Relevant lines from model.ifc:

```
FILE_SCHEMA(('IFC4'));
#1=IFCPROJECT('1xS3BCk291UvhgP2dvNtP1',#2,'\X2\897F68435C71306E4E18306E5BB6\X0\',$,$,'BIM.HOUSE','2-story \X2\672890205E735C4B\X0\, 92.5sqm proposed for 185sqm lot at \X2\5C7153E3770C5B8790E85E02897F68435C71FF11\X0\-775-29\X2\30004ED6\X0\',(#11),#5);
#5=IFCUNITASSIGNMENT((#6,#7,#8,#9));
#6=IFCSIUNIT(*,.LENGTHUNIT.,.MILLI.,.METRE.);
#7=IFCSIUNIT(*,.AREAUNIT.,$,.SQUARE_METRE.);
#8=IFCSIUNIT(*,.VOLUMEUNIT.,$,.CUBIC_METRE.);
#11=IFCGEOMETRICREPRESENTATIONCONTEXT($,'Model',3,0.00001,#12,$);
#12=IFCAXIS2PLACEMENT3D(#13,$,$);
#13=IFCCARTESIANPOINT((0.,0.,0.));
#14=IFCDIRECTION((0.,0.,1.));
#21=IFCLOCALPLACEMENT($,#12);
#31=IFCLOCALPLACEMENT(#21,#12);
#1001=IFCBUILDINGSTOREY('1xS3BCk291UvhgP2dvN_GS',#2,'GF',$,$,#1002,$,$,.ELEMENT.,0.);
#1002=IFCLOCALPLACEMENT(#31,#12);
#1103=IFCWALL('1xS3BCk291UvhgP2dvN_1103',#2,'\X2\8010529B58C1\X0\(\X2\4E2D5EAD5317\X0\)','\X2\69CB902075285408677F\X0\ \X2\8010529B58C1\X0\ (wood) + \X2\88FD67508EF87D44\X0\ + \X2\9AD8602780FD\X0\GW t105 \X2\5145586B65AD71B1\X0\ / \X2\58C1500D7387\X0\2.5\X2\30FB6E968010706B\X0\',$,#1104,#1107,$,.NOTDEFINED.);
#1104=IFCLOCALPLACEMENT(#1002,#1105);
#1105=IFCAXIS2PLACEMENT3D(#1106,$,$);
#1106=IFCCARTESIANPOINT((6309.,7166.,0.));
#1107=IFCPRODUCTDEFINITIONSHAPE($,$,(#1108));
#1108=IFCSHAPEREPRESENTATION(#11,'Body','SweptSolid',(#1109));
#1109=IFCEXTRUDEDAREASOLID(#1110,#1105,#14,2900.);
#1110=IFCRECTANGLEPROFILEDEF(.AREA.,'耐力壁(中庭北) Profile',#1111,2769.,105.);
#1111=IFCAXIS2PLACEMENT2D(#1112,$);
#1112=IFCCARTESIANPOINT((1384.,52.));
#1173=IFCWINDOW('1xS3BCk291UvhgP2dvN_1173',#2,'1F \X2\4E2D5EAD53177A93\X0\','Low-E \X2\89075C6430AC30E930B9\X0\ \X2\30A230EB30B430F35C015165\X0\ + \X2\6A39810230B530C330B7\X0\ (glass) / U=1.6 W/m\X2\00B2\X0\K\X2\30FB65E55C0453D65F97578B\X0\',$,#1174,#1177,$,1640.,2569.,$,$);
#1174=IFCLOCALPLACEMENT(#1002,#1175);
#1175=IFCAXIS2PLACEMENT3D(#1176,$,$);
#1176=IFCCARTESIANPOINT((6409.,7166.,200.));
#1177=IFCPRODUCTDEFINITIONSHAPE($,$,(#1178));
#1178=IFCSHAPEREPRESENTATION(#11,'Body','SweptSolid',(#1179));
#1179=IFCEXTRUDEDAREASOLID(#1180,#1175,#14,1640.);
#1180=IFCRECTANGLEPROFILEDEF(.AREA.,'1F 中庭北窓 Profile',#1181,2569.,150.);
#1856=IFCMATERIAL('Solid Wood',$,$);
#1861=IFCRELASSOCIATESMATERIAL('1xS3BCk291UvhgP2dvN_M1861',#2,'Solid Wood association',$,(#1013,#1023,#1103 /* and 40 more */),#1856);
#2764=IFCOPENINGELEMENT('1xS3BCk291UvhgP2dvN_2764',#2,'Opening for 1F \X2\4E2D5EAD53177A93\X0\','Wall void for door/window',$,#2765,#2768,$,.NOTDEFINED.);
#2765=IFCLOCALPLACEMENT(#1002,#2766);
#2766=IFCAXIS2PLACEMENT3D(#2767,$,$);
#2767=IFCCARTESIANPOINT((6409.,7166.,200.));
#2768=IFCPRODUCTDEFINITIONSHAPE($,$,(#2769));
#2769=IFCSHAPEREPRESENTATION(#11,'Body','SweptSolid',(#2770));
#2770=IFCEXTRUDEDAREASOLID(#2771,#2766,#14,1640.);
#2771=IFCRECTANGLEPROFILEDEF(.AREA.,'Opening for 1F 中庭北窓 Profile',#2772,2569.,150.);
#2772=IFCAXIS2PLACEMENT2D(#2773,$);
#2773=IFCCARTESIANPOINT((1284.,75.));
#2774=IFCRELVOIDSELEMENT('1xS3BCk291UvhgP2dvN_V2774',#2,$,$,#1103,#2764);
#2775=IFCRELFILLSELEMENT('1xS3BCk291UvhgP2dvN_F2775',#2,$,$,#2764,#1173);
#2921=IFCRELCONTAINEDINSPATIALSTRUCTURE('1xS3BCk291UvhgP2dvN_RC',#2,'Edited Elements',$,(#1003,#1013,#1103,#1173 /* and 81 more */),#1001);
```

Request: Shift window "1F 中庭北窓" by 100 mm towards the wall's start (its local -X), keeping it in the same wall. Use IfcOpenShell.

```python
import ifcopenshell
import ifcopenshell.api.geometry
import ifcopenshell.util.placement

model = ifcopenshell.open("model.ifc")

window = model.by_guid("1xS3BCk291UvhgP2dvN_1173")
opening = window.FillsVoids[0].RelatingOpeningElement
wall = opening.VoidsElements[0].RelatingBuildingElement

wall_matrix = ifcopenshell.util.placement.get_local_placement(wall.ObjectPlacement)
shift = wall_matrix[:3, 0] * -100.0
before = ifcopenshell.util.placement.get_local_placement(window.ObjectPlacement)[:3, 3].copy()

# The window is not placed relative to its opening, so move both.
for product in (opening, window):
    matrix = ifcopenshell.util.placement.get_local_placement(product.ObjectPlacement)
    matrix[:3, 3] += shift
    ifcopenshell.api.geometry.edit_object_placement(model, product=product, matrix=matrix, is_si=False)

after = ifcopenshell.util.placement.get_local_placement(window.ObjectPlacement)[:3, 3]
print("window moved by", (after - before).round(3) + 0.0)

model.write("model_v2.ifc")
```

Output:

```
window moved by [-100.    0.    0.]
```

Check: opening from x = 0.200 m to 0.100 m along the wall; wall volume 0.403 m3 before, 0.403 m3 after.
